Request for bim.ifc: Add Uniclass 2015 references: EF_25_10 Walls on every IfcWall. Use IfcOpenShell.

First a look at what the model holds.

```python
import ifcopenshell

model = ifcopenshell.open("bim.ifc")
print(model.schema)
print("classifications:", [c.Name for c in model.by_type("IfcClassification")])
for ifc_class in ("IfcDoor", "IfcRoof", "IfcStair", "IfcWall", "IfcWindow"):
    print(ifc_class, len(model.by_type(ifc_class)))
```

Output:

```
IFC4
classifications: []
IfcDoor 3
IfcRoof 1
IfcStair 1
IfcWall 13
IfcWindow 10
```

```python
import ifcopenshell
import ifcopenshell.api.classification

model = ifcopenshell.open("bim.ifc")

system = ifcopenshell.api.classification.add_classification(model, classification="Uniclass 2015")

codes = {
    "IfcWall": ("EF_25_10", "Walls"),
}
for ifc_class, (code, name) in codes.items():
    products = model.by_type(ifc_class)
    ifcopenshell.api.classification.add_reference(
        model, products=products, classification=system, identification=code, name=name
    )
    print(code, len(products))

model.write("bim_edited.ifc")
```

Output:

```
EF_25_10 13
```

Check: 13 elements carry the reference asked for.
